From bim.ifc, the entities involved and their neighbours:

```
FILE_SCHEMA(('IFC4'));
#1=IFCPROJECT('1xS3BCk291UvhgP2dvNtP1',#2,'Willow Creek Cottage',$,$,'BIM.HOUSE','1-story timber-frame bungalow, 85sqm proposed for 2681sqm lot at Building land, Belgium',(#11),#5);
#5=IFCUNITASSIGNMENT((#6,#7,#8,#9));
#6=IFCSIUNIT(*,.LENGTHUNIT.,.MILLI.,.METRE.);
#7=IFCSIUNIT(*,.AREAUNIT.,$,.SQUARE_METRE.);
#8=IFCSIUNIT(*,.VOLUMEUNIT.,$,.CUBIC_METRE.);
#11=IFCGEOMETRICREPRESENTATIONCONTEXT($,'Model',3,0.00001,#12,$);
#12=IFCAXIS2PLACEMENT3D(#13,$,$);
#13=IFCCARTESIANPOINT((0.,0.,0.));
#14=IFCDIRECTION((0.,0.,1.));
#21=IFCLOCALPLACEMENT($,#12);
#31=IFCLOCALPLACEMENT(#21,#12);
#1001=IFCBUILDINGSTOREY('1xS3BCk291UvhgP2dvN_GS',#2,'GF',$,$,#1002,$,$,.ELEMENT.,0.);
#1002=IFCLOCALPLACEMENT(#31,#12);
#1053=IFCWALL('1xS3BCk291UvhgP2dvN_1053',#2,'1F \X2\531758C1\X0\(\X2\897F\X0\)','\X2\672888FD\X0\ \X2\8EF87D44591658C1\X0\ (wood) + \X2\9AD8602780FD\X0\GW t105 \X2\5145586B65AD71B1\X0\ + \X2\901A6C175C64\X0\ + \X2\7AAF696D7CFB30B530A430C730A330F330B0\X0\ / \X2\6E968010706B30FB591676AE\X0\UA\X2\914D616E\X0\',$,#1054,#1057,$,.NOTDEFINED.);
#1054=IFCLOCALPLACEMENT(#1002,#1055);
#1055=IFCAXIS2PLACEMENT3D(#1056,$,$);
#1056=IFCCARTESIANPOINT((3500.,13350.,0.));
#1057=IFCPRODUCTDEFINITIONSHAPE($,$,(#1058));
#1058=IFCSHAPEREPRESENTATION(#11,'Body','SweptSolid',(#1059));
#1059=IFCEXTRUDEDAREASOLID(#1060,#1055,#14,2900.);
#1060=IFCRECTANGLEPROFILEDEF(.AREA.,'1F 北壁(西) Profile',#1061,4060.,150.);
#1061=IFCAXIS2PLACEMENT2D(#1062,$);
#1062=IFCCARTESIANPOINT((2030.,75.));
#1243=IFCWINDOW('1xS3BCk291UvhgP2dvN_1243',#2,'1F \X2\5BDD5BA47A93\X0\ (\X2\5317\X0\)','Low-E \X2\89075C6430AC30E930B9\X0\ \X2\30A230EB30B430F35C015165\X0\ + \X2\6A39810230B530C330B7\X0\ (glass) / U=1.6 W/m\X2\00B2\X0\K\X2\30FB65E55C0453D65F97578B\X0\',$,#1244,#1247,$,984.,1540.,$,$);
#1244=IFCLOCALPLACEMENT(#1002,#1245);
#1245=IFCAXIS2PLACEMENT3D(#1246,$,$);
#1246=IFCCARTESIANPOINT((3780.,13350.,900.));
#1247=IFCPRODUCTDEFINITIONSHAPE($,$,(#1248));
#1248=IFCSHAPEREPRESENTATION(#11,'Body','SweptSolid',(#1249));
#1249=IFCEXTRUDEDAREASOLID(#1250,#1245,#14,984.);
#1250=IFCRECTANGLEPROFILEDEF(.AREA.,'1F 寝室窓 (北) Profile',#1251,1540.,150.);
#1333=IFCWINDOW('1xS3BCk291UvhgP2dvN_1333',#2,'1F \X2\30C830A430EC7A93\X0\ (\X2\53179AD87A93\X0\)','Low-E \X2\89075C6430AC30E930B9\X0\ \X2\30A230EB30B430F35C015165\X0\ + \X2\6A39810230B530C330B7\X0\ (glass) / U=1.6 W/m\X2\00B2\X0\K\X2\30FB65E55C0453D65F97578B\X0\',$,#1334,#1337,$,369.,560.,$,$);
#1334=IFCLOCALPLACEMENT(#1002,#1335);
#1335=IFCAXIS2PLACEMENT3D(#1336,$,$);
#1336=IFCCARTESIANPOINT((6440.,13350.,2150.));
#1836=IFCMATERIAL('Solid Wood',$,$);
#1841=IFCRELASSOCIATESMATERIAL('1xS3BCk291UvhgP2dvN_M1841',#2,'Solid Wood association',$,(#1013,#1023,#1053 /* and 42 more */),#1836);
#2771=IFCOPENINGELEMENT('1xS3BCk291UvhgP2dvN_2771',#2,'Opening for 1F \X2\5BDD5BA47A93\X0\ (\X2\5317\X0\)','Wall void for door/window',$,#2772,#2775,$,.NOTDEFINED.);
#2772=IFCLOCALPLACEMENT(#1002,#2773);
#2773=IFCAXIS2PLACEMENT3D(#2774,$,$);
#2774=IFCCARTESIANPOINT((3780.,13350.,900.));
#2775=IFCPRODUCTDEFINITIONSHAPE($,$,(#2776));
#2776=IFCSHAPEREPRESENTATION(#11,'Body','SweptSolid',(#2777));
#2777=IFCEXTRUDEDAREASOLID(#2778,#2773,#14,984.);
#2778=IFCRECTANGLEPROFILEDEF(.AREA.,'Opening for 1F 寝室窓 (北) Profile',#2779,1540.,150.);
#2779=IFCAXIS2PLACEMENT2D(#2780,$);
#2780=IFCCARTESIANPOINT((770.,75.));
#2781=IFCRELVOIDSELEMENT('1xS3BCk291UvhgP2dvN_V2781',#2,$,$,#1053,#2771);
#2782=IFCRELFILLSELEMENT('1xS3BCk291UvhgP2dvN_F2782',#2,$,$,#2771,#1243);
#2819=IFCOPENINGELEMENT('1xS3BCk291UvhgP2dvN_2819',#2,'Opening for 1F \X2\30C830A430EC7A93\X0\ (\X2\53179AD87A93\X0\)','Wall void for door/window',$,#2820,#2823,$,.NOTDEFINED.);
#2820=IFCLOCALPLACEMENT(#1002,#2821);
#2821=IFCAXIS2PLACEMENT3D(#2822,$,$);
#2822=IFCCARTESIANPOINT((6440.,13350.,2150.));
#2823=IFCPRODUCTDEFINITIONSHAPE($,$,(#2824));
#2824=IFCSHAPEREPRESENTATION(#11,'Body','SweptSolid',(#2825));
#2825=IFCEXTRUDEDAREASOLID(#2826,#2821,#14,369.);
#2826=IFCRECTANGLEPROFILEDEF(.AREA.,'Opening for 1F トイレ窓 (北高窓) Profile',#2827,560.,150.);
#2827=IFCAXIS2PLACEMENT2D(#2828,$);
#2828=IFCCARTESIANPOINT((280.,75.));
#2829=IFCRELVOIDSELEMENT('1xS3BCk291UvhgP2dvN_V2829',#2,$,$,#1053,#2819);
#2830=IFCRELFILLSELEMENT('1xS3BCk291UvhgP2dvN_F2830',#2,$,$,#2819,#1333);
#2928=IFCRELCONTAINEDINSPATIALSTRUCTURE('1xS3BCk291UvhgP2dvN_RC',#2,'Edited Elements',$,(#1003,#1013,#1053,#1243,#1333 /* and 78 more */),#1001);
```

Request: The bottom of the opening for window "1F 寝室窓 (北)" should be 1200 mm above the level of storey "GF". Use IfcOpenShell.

```python
import numpy as np
import ifcopenshell
import ifcopenshell.api.geometry
import ifcopenshell.geom
import ifcopenshell.util.element
import ifcopenshell.util.placement
import ifcopenshell.util.shape
import ifcopenshell.util.unit

model = ifcopenshell.open("bim.ifc")
unit_scale = ifcopenshell.util.unit.calculate_unit_scale(model)

window = model.by_id(1243)
opening = window.FillsVoids[0].RelatingOpeningElement
storey = ifcopenshell.util.element.get_container(window, ifc_class="IfcBuildingStorey")
level = ifcopenshell.util.placement.get_local_placement(storey.ObjectPlacement)[2, 3]

# The opening's origin need not be at the sill, so measure its lowest point.
shape = ifcopenshell.geom.create_shape(ifcopenshell.geom.settings(), opening)
bottom = ifcopenshell.util.shape.get_shape_bottom_elevation(shape, shape.geometry) / unit_scale
dz = level + 1.2 / unit_scale - bottom

shift = np.array([0.0, 0.0, dz])
# The window is not placed relative to its opening, so move both.
for product in (opening, window):
    matrix = ifcopenshell.util.placement.get_local_placement(product.ObjectPlacement)
    matrix[:3, 3] += shift
    ifcopenshell.api.geometry.edit_object_placement(model, product=product, matrix=matrix, is_si=False)

print(f"moved by {dz * unit_scale:+.3f} m")

model.write("bim-out.ifc")
```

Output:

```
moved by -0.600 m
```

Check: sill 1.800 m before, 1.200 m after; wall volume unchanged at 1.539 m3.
